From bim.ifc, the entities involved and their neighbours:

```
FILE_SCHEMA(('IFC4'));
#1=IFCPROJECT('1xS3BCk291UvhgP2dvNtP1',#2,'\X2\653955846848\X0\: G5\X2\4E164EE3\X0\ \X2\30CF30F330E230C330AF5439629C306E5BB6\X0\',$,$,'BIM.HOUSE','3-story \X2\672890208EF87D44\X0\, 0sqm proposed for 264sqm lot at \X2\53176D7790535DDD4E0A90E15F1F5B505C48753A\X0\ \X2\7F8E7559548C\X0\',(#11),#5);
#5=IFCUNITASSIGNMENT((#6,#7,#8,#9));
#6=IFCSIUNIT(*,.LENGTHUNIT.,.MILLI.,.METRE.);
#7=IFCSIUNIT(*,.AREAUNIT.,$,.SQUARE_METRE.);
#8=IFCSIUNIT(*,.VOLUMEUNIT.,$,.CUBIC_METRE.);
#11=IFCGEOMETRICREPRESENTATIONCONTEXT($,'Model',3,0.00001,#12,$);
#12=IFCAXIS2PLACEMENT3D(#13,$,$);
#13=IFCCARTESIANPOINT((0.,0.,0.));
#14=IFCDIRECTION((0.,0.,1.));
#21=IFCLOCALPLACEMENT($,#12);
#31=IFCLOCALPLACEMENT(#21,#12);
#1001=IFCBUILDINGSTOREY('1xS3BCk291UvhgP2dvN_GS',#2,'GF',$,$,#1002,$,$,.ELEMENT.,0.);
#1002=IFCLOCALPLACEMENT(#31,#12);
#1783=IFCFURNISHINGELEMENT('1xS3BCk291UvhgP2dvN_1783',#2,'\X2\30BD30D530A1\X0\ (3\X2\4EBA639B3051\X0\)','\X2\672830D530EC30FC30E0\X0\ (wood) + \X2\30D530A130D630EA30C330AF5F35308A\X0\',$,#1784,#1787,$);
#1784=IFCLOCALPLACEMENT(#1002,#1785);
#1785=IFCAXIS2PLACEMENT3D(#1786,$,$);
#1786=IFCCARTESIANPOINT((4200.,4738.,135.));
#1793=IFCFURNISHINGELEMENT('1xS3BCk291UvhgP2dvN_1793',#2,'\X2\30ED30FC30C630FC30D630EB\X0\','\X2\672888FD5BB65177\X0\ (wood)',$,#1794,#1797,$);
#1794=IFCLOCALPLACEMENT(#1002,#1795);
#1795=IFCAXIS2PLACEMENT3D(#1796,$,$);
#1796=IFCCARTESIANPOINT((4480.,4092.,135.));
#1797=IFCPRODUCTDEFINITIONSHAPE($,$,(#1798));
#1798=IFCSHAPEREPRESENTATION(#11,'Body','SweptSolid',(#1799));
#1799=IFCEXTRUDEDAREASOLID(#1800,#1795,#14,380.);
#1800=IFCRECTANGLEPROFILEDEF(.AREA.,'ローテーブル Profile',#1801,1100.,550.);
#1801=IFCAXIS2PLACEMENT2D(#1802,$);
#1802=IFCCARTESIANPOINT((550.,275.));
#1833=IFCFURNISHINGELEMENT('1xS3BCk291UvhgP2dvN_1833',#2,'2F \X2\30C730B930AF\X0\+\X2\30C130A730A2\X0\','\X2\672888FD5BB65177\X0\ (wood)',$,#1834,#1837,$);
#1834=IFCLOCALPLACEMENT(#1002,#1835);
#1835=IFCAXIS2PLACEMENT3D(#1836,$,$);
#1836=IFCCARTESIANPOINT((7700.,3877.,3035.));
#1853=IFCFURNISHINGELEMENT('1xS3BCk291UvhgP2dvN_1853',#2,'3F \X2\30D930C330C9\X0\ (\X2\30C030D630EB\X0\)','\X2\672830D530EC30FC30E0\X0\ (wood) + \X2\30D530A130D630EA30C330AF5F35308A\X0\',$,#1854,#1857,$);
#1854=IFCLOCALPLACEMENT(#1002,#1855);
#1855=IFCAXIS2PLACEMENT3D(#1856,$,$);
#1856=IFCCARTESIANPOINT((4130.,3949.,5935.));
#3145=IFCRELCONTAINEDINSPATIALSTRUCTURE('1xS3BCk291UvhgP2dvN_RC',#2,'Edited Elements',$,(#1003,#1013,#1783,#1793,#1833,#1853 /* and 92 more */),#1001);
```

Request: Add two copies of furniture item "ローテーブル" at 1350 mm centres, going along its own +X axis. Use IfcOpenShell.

```python
import ifcopenshell
import ifcopenshell.api.geometry
import ifcopenshell.api.root
import ifcopenshell.util.element
import ifcopenshell.util.placement

model = ifcopenshell.open("bim.ifc")


def reuse_history(source, copy):
    """copy_class also copies each property set's owner history, people and application; keep the originals."""
    for rel in copy.IsDefinedBy:
        if rel.is_a("IfcRelDefinesByProperties") and (history := rel.RelatingPropertyDefinition.OwnerHistory):
            rel.RelatingPropertyDefinition.OwnerHistory = source.OwnerHistory
            ifcopenshell.util.element.remove_deep2(model, history)


source = model.by_id(1793)
base = ifcopenshell.util.placement.get_local_placement(source.ObjectPlacement)
step = base[:3, 0] * 1350.0

for i in range(1, 3):
    copy = ifcopenshell.api.root.copy_class(model, product=source)
    copy.Representation = ifcopenshell.util.element.copy_deep(
        model, source.Representation, exclude=["IfcGeometricRepresentationContext", "IfcRepresentationMap"]
    )
    reuse_history(source, copy)
    matrix = base.copy()
    matrix[:3, 3] += i * step
    print("added at", matrix[:3, 3].round(3) + 0.0)
    ifcopenshell.api.geometry.edit_object_placement(model, product=copy, matrix=matrix, is_si=False)

model.write("bim_v2.ifc")
```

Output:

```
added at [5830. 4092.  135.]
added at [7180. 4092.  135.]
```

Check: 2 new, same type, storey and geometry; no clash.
